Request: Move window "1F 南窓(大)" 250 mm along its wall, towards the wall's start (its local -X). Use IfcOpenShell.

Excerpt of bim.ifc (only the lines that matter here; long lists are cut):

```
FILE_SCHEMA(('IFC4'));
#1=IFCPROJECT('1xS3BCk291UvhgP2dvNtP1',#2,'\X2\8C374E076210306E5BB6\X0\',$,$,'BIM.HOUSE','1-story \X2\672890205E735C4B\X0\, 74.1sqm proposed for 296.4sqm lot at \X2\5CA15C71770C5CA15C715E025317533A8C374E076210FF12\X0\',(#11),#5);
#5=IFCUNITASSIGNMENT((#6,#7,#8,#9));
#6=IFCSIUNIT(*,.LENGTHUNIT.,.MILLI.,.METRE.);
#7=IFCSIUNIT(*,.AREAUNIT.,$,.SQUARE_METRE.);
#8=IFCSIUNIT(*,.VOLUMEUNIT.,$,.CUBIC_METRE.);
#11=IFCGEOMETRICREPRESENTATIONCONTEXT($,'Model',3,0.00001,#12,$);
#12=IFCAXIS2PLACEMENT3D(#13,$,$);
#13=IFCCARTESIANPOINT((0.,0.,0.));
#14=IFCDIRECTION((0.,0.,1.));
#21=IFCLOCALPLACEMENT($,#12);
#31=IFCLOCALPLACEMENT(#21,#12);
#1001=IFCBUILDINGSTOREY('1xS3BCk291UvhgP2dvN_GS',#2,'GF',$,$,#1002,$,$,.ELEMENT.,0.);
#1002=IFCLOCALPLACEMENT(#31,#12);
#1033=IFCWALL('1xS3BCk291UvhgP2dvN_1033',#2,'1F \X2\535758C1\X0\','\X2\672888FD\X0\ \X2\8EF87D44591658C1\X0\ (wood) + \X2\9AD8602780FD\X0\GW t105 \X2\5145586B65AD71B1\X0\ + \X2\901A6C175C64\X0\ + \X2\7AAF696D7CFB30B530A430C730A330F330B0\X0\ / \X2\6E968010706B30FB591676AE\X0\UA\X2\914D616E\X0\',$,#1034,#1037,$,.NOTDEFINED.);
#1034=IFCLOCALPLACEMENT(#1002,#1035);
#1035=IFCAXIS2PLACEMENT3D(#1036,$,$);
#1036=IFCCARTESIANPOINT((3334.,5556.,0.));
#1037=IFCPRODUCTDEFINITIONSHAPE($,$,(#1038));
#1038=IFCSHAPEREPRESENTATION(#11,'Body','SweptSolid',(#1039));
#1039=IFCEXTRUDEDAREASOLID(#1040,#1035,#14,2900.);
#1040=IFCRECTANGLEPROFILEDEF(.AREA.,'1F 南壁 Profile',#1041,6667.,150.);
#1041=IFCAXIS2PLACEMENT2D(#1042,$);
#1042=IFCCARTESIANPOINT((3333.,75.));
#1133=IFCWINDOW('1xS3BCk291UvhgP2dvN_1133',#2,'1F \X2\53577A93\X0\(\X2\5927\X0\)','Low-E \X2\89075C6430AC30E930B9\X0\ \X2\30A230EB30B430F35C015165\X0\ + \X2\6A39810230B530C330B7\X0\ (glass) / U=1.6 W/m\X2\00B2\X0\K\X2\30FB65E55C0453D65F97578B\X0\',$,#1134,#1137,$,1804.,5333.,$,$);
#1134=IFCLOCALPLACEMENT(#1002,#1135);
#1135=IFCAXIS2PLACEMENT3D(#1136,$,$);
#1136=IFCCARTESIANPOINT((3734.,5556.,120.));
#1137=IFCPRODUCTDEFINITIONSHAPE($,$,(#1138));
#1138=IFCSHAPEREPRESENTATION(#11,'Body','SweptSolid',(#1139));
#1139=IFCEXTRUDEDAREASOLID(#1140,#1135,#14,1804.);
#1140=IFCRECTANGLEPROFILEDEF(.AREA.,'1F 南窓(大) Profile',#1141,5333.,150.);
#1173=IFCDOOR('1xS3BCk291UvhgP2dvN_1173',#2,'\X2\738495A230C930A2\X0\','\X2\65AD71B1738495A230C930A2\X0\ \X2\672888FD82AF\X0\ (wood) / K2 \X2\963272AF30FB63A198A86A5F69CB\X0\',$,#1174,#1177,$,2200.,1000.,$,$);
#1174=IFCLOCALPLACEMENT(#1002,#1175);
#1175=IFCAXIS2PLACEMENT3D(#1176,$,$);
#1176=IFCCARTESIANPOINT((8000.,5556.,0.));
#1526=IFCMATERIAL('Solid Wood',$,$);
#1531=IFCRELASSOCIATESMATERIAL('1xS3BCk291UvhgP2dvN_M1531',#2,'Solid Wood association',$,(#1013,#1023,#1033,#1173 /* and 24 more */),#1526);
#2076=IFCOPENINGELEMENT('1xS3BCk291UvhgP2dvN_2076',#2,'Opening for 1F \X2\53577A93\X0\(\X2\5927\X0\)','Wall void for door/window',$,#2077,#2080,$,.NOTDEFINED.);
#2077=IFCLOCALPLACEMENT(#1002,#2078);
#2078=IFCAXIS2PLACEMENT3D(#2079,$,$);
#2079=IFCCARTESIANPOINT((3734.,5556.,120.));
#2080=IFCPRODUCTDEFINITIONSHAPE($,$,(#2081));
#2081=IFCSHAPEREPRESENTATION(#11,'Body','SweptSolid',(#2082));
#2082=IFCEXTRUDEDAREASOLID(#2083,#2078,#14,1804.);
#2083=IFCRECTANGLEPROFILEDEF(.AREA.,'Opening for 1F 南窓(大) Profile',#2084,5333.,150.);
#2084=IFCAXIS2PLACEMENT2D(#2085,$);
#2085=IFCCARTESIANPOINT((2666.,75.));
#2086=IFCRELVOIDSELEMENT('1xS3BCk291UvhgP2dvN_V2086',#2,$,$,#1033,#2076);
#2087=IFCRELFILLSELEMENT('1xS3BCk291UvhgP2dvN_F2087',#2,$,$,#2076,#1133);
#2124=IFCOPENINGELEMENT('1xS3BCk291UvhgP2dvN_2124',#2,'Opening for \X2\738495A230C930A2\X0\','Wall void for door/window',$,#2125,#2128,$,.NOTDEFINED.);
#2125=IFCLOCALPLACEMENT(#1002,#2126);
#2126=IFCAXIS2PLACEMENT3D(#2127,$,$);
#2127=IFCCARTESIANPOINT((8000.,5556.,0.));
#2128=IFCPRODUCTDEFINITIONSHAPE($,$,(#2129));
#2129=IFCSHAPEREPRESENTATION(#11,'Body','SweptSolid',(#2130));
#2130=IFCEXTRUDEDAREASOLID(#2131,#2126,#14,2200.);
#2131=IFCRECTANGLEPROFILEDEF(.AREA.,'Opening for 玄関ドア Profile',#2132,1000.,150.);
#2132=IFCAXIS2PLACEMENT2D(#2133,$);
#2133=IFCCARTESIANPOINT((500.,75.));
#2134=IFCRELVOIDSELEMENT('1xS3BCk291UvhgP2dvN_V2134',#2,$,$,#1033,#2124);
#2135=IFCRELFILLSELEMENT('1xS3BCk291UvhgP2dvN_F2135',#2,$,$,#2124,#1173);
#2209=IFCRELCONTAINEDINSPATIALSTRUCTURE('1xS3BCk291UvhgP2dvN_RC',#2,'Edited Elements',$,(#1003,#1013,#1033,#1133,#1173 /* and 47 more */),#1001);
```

```python
import ifcopenshell
import ifcopenshell.api.geometry
import ifcopenshell.util.placement
import ifcopenshell.util.unit

model = ifcopenshell.open("bim.ifc")
unit_scale = ifcopenshell.util.unit.calculate_unit_scale(model)

window = model.by_id(1133)
opening = window.FillsVoids[0].RelatingOpeningElement
wall = opening.VoidsElements[0].RelatingBuildingElement

wall_matrix = ifcopenshell.util.placement.get_local_placement(wall.ObjectPlacement)
shift = wall_matrix[:3, 0] * -0.25 / unit_scale
before = ifcopenshell.util.placement.get_local_placement(window.ObjectPlacement)[:3, 3].copy()

# The window is not placed relative to its opening, so move both.
for product in (opening, window):
    matrix = ifcopenshell.util.placement.get_local_placement(product.ObjectPlacement)
    matrix[:3, 3] += shift
    ifcopenshell.api.geometry.edit_object_placement(model, product=product, matrix=matrix, is_si=False)

after = ifcopenshell.util.placement.get_local_placement(window.ObjectPlacement)[:3, 3]
print("window moved by", (after - before).round(3) + 0.0)

model.write("bim_updated.ifc")
```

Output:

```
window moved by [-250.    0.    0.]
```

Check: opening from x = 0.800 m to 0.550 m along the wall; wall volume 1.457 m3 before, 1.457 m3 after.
